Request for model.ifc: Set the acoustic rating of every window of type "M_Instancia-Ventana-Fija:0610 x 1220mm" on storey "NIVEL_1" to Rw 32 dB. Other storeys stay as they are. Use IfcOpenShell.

First a look at what the model holds.

```python
import ifcopenshell
import ifcopenshell.util.element

model = ifcopenshell.open("model.ifc")
print(model.schema)
storey = next(s for s in model.by_type("IfcBuildingStorey") if s.Name == "NIVEL_1")
windows = [e for e in ifcopenshell.util.element.get_decomposition(storey) if e.is_a("IfcWindow")]
seen = {}
for e in windows:
    element_type = ifcopenshell.util.element.get_type(e)
    key = (element_type.Name if element_type != e and element_type else None, ifcopenshell.util.element.get_pset(e, "Pset_WindowCommon", "AcousticRating"))
    seen[key] = seen.get(key, 0) + 1
for (name, value), count in sorted(seen.items(), key=str):
    print(count, "x", name, "|", value)
```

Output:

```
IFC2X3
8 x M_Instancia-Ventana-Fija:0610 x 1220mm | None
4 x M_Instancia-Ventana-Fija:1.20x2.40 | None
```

```python
import ifcopenshell
import ifcopenshell.api.pset
import ifcopenshell.util.element

model = ifcopenshell.open("model.ifc")

storey = next(s for s in model.by_type("IfcBuildingStorey") if s.Name == "NIVEL_1")
windows = [e for e in ifcopenshell.util.element.get_decomposition(storey) if e.is_a("IfcWindow")]

count = 0
for e in windows:
    element_type = ifcopenshell.util.element.get_type(e)
    if element_type in (None, e) or element_type.Name != "M_Instancia-Ventana-Fija:0610 x 1220mm":
        continue
    # add_pset returns the element's existing set when there is one.
    pset = ifcopenshell.api.pset.add_pset(model, product=e, name="Pset_WindowCommon")
    ifcopenshell.api.pset.edit_pset(model, pset=pset, properties={"AcousticRating": "Rw 32 dB"})
    count += 1

print(count, "windows updated")

model.write("model-out.ifc")
```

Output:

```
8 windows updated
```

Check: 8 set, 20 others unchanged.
